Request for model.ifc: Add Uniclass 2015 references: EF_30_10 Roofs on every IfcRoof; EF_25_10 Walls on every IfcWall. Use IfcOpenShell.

First a look at what the model holds.

```python
import ifcopenshell

model = ifcopenshell.open("model.ifc")
print(model.schema)
print("classifications:", [c.Name for c in model.by_type("IfcClassification")])
for ifc_class in ("IfcDoor", "IfcRoof", "IfcStair", "IfcWall", "IfcWindow"):
    print(ifc_class, len(model.by_type(ifc_class)))
```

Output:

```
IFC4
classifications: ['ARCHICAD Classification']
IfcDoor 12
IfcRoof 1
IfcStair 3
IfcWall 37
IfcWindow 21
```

```python
import ifcopenshell
import ifcopenshell.api.classification

model = ifcopenshell.open("model.ifc")

system = ifcopenshell.api.classification.add_classification(model, classification="Uniclass 2015")

codes = {
    "IfcRoof": ("EF_30_10", "Roofs"),
    "IfcWall": ("EF_25_10", "Walls"),
}
for ifc_class, (code, name) in codes.items():
    products = model.by_type(ifc_class)
    ifcopenshell.api.classification.add_reference(
        model, products=products, classification=system, identification=code, name=name
    )
    print(code, len(products))

model.write("model_updated.ifc")
```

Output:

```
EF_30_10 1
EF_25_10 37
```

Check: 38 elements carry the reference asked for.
